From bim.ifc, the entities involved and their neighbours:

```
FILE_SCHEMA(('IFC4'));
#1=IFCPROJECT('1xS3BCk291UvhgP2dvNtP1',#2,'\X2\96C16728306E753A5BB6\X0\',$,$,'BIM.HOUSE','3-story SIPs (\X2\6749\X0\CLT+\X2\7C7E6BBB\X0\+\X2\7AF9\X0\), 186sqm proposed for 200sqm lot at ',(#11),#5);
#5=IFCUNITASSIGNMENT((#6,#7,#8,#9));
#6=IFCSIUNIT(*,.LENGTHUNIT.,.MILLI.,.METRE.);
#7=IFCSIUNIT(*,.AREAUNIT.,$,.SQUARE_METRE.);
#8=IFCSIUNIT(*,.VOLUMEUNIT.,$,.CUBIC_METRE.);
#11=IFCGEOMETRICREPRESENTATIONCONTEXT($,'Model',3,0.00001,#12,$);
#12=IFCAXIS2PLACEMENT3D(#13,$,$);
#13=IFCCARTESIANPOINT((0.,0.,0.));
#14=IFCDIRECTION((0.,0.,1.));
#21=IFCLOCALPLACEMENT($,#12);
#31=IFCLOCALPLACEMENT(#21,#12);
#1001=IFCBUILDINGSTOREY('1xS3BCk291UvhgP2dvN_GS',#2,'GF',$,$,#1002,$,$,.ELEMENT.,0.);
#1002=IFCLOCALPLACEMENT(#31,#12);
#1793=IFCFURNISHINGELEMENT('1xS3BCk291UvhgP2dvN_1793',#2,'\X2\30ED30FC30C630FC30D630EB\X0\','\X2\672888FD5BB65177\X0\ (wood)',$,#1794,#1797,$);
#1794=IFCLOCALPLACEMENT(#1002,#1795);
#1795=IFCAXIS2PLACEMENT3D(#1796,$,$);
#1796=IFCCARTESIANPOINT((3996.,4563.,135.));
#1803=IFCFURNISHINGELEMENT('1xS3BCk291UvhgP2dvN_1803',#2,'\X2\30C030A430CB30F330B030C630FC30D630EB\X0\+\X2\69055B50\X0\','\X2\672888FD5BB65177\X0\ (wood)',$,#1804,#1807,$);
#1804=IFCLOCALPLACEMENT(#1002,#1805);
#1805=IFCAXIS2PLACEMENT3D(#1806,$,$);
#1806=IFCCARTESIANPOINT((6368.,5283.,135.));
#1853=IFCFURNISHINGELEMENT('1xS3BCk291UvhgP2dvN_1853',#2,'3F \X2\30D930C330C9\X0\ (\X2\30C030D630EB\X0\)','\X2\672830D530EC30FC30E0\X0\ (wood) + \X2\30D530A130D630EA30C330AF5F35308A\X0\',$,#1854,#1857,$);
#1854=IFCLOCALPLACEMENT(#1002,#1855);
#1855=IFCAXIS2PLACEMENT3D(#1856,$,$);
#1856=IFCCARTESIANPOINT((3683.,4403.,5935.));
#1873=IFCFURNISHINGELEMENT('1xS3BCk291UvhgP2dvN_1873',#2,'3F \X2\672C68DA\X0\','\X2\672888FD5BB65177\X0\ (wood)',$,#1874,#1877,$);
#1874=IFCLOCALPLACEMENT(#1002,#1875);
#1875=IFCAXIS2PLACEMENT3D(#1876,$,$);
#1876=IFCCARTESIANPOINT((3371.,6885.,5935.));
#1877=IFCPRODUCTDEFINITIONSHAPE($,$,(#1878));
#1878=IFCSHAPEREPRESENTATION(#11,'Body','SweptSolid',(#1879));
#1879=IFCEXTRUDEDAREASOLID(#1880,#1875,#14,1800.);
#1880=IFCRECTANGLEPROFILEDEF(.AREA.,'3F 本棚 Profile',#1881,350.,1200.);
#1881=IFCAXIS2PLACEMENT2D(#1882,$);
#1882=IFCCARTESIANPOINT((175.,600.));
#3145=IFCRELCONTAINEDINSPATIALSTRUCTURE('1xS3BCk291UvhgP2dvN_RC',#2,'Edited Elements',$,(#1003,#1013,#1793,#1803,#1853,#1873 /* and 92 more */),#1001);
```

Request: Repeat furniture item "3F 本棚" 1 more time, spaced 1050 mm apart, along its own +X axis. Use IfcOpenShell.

```python
import ifcopenshell
import ifcopenshell.api.geometry
import ifcopenshell.api.root
import ifcopenshell.util.element
import ifcopenshell.util.placement
import ifcopenshell.util.unit

model = ifcopenshell.open("bim.ifc")
unit_scale = ifcopenshell.util.unit.calculate_unit_scale(model)


def reuse_history(source, copy):
    """copy_class also copies each property set's owner history, people and application; keep the originals."""
    for rel in copy.IsDefinedBy:
        if rel.is_a("IfcRelDefinesByProperties") and (history := rel.RelatingPropertyDefinition.OwnerHistory):
            rel.RelatingPropertyDefinition.OwnerHistory = source.OwnerHistory
            ifcopenshell.util.element.remove_deep2(model, history)


source = model.by_guid("1xS3BCk291UvhgP2dvN_1873")
base = ifcopenshell.util.placement.get_local_placement(source.ObjectPlacement)
step = base[:3, 0] * 1.05 / unit_scale

for i in range(1, 2):
    copy = ifcopenshell.api.root.copy_class(model, product=source)
    copy.Representation = ifcopenshell.util.element.copy_deep(
        model, source.Representation, exclude=["IfcGeometricRepresentationContext", "IfcRepresentationMap"]
    )
    reuse_history(source, copy)
    matrix = base.copy()
    matrix[:3, 3] += i * step
    print("added at", matrix[:3, 3].round(3) + 0.0)
    ifcopenshell.api.geometry.edit_object_placement(model, product=copy, matrix=matrix, is_si=False)

model.write("bim_rev.ifc")
```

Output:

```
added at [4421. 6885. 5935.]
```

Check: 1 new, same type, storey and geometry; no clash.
